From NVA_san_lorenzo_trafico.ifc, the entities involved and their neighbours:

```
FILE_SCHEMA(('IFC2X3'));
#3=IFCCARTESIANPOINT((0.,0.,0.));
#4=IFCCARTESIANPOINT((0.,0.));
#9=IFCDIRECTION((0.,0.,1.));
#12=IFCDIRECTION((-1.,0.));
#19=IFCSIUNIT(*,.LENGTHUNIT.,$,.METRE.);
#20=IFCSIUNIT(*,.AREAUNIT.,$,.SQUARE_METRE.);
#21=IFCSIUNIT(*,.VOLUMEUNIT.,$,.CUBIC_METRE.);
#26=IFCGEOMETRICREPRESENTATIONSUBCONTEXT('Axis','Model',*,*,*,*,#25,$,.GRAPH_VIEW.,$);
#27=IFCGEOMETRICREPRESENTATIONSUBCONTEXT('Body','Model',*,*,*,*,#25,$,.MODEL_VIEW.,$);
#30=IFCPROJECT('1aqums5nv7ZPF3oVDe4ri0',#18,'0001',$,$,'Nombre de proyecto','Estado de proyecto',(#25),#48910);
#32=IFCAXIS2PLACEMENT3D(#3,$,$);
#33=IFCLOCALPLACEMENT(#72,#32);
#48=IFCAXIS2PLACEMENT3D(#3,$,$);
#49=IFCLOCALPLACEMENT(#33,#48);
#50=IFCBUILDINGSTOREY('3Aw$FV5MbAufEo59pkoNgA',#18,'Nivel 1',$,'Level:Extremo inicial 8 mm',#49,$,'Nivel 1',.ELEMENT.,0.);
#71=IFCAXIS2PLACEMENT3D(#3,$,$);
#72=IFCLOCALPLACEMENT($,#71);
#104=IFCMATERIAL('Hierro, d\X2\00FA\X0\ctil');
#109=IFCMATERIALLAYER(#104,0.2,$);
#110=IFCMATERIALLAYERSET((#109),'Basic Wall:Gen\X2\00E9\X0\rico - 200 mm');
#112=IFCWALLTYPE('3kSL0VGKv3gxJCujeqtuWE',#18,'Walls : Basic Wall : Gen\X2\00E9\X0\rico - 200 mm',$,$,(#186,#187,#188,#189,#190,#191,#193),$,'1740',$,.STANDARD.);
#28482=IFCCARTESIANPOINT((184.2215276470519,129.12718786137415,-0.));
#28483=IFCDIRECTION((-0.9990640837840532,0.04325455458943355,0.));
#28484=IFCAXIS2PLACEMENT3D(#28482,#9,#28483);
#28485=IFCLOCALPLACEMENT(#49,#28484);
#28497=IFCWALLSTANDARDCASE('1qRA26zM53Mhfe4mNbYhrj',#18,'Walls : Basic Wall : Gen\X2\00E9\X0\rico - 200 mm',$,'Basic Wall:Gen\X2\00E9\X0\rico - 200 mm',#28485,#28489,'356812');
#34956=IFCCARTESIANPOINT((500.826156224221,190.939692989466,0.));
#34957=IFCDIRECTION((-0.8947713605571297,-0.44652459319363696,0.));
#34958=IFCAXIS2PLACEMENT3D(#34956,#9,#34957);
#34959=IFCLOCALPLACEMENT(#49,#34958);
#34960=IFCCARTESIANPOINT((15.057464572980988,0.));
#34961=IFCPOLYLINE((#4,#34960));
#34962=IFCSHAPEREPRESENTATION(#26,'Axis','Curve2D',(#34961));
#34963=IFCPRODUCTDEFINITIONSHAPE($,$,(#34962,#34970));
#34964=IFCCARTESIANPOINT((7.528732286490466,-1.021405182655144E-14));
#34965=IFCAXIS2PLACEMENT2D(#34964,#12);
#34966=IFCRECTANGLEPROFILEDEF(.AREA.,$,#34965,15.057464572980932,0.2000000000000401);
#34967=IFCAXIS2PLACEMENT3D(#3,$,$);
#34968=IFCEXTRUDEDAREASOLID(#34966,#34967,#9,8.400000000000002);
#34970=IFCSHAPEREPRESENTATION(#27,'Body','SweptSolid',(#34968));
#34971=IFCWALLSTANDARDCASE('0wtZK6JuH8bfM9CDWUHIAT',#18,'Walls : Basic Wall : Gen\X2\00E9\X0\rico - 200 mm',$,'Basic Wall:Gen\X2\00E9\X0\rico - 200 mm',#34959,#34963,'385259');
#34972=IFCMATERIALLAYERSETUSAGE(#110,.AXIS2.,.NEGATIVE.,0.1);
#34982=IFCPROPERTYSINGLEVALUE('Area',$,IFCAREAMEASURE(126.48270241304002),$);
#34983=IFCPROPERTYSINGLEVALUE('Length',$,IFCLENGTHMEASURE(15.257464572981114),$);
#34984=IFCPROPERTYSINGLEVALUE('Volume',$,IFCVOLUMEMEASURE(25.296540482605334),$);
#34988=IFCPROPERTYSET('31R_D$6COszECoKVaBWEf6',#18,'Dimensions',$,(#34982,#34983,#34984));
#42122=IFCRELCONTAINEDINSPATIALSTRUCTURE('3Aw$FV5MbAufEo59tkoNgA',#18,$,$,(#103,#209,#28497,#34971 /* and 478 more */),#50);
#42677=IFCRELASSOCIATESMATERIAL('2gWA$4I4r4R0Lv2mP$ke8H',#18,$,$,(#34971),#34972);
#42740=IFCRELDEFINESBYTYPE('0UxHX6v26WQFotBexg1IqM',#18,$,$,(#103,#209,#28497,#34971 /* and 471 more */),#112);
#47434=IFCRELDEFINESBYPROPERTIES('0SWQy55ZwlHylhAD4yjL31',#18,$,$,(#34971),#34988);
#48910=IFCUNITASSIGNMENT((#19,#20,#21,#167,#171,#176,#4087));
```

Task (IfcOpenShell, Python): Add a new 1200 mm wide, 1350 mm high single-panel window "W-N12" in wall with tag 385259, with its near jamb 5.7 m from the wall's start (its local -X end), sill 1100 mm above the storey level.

```python
import numpy as np
import ifcopenshell
import ifcopenshell.api.feature
import ifcopenshell.api.geometry
import ifcopenshell.api.pset
import ifcopenshell.api.root
import ifcopenshell.api.spatial
import ifcopenshell.api.type
import ifcopenshell.geom
import ifcopenshell.util.element
import ifcopenshell.util.placement
import ifcopenshell.util.representation
import ifcopenshell.util.shape
import ifcopenshell.util.unit

model = ifcopenshell.open("NVA_san_lorenzo_trafico.ifc")
unit_scale = ifcopenshell.util.unit.calculate_unit_scale(model)
area_scale = ifcopenshell.util.unit.calculate_unit_scale(model, "AREAUNIT")
volume_scale = ifcopenshell.util.unit.calculate_unit_scale(model, "VOLUMEUNIT")
settings = ifcopenshell.geom.settings()


def volume(element):
    """Net volume in cubic metres, openings subtracted."""
    shape = ifcopenshell.geom.create_shape(settings, element)
    return ifcopenshell.util.shape.get_volume(shape.geometry)


wall = model.by_id(34971)
storey = ifcopenshell.util.element.get_container(wall, ifc_class="IfcBuildingStorey")
context = ifcopenshell.util.representation.get_context(model, "Model", "Body", "MODEL_VIEW")
before = volume(wall)

width, height, from_end, sill = 1.2, 1.35, 5.7, 1.1  # metres

# The wall runs along its own X axis, and the end named is its -X end.
wall_shape = ifcopenshell.geom.create_shape(settings, wall)
x, y, z = ifcopenshell.util.shape.get_vertices(wall_shape.geometry).T
start = x.min() + from_end
face, thickness = float(y.min()), float(y.max() - y.min())
wall_matrix = ifcopenshell.util.placement.get_local_placement(wall.ObjectPlacement)
level = ifcopenshell.util.placement.get_local_placement(storey.ObjectPlacement)[2, 3]


def in_wall(x, y):
    """Placement at x, y metres in the wall's axes, at sill height."""
    matrix = wall_matrix.copy()
    matrix[:, 3] = wall_matrix @ np.array([x / unit_scale, y / unit_scale, 0.0, 1.0])
    matrix[2, 3] = level + sill / unit_scale
    return matrix


# Opening: a box that overshoots both wall faces by 50 mm.
opening = ifcopenshell.api.root.create_entity(model, ifc_class="IfcOpeningElement")
box = ifcopenshell.api.geometry.add_wall_representation(
    model, context=context, length=width, height=height, thickness=thickness + 0.1
)
ifcopenshell.api.geometry.assign_representation(model, product=opening, representation=box)
ifcopenshell.api.geometry.edit_object_placement(model, product=opening, matrix=in_wall(start, face - 0.05), is_si=False)
ifcopenshell.api.feature.add_feature(model, feature=opening, element=wall)

window = ifcopenshell.api.root.create_entity(model, ifc_class="IfcWindow", name="W-N12")
window.OverallWidth, window.OverallHeight = width / unit_scale, height / unit_scale
body = ifcopenshell.api.geometry.add_window_representation(
    model,
    context=context,
    overall_width=window.OverallWidth,
    overall_height=window.OverallHeight,
    partition_type="SINGLE_PANEL",
)
ifcopenshell.api.geometry.assign_representation(model, product=window, representation=body)
ifcopenshell.api.spatial.assign_container(model, products=[window], relating_structure=storey)
fills = ifcopenshell.api.feature.add_filling(model, opening=opening, element=window)
fills.OwnerHistory = window.OwnerHistory  # required in IFC2X3

# IFC2X3 keeps the operation on the window style.
style = ifcopenshell.api.root.create_entity(model, ifc_class="IfcWindowStyle", name="W-N12")
style.OperationType, style.ConstructionType = "SINGLE_PANEL", "NOTDEFINED"
style.ParameterTakesPrecedence = style.Sizeable = False
ifcopenshell.api.type.assign_type(model, related_objects=[window], relating_type=style)

# Centre the window in the wall's thickness.
ifcopenshell.api.geometry.edit_object_placement(model, product=window, matrix=in_wall(start, face), is_si=False)
window_shape = ifcopenshell.geom.create_shape(settings, window)
depth = ifcopenshell.util.shape.get_vertices(window_shape.geometry)[:, 1]
offset = face + thickness / 2 - (depth.min() + depth.max()) / 2
ifcopenshell.api.geometry.edit_object_placement(model, product=window, matrix=in_wall(start, offset), is_si=False)

after = volume(wall)

# Update the wall's stored quantities.
pset = model.by_id(ifcopenshell.util.element.get_pset(wall, "Dimensions", should_inherit=False)["id"])
ifcopenshell.api.pset.edit_pset(model, pset=pset, properties={
    "Area": model.create_entity("IfcAreaMeasure", after / thickness / area_scale),
    "Volume": model.create_entity("IfcVolumeMeasure", after / volume_scale),
})

print(f"wall volume {before:.3f} -> {after:.3f} m3")

model.write("NVA_san_lorenzo_trafico-out.ifc")
```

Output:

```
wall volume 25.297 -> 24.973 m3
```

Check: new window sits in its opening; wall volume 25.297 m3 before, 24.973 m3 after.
